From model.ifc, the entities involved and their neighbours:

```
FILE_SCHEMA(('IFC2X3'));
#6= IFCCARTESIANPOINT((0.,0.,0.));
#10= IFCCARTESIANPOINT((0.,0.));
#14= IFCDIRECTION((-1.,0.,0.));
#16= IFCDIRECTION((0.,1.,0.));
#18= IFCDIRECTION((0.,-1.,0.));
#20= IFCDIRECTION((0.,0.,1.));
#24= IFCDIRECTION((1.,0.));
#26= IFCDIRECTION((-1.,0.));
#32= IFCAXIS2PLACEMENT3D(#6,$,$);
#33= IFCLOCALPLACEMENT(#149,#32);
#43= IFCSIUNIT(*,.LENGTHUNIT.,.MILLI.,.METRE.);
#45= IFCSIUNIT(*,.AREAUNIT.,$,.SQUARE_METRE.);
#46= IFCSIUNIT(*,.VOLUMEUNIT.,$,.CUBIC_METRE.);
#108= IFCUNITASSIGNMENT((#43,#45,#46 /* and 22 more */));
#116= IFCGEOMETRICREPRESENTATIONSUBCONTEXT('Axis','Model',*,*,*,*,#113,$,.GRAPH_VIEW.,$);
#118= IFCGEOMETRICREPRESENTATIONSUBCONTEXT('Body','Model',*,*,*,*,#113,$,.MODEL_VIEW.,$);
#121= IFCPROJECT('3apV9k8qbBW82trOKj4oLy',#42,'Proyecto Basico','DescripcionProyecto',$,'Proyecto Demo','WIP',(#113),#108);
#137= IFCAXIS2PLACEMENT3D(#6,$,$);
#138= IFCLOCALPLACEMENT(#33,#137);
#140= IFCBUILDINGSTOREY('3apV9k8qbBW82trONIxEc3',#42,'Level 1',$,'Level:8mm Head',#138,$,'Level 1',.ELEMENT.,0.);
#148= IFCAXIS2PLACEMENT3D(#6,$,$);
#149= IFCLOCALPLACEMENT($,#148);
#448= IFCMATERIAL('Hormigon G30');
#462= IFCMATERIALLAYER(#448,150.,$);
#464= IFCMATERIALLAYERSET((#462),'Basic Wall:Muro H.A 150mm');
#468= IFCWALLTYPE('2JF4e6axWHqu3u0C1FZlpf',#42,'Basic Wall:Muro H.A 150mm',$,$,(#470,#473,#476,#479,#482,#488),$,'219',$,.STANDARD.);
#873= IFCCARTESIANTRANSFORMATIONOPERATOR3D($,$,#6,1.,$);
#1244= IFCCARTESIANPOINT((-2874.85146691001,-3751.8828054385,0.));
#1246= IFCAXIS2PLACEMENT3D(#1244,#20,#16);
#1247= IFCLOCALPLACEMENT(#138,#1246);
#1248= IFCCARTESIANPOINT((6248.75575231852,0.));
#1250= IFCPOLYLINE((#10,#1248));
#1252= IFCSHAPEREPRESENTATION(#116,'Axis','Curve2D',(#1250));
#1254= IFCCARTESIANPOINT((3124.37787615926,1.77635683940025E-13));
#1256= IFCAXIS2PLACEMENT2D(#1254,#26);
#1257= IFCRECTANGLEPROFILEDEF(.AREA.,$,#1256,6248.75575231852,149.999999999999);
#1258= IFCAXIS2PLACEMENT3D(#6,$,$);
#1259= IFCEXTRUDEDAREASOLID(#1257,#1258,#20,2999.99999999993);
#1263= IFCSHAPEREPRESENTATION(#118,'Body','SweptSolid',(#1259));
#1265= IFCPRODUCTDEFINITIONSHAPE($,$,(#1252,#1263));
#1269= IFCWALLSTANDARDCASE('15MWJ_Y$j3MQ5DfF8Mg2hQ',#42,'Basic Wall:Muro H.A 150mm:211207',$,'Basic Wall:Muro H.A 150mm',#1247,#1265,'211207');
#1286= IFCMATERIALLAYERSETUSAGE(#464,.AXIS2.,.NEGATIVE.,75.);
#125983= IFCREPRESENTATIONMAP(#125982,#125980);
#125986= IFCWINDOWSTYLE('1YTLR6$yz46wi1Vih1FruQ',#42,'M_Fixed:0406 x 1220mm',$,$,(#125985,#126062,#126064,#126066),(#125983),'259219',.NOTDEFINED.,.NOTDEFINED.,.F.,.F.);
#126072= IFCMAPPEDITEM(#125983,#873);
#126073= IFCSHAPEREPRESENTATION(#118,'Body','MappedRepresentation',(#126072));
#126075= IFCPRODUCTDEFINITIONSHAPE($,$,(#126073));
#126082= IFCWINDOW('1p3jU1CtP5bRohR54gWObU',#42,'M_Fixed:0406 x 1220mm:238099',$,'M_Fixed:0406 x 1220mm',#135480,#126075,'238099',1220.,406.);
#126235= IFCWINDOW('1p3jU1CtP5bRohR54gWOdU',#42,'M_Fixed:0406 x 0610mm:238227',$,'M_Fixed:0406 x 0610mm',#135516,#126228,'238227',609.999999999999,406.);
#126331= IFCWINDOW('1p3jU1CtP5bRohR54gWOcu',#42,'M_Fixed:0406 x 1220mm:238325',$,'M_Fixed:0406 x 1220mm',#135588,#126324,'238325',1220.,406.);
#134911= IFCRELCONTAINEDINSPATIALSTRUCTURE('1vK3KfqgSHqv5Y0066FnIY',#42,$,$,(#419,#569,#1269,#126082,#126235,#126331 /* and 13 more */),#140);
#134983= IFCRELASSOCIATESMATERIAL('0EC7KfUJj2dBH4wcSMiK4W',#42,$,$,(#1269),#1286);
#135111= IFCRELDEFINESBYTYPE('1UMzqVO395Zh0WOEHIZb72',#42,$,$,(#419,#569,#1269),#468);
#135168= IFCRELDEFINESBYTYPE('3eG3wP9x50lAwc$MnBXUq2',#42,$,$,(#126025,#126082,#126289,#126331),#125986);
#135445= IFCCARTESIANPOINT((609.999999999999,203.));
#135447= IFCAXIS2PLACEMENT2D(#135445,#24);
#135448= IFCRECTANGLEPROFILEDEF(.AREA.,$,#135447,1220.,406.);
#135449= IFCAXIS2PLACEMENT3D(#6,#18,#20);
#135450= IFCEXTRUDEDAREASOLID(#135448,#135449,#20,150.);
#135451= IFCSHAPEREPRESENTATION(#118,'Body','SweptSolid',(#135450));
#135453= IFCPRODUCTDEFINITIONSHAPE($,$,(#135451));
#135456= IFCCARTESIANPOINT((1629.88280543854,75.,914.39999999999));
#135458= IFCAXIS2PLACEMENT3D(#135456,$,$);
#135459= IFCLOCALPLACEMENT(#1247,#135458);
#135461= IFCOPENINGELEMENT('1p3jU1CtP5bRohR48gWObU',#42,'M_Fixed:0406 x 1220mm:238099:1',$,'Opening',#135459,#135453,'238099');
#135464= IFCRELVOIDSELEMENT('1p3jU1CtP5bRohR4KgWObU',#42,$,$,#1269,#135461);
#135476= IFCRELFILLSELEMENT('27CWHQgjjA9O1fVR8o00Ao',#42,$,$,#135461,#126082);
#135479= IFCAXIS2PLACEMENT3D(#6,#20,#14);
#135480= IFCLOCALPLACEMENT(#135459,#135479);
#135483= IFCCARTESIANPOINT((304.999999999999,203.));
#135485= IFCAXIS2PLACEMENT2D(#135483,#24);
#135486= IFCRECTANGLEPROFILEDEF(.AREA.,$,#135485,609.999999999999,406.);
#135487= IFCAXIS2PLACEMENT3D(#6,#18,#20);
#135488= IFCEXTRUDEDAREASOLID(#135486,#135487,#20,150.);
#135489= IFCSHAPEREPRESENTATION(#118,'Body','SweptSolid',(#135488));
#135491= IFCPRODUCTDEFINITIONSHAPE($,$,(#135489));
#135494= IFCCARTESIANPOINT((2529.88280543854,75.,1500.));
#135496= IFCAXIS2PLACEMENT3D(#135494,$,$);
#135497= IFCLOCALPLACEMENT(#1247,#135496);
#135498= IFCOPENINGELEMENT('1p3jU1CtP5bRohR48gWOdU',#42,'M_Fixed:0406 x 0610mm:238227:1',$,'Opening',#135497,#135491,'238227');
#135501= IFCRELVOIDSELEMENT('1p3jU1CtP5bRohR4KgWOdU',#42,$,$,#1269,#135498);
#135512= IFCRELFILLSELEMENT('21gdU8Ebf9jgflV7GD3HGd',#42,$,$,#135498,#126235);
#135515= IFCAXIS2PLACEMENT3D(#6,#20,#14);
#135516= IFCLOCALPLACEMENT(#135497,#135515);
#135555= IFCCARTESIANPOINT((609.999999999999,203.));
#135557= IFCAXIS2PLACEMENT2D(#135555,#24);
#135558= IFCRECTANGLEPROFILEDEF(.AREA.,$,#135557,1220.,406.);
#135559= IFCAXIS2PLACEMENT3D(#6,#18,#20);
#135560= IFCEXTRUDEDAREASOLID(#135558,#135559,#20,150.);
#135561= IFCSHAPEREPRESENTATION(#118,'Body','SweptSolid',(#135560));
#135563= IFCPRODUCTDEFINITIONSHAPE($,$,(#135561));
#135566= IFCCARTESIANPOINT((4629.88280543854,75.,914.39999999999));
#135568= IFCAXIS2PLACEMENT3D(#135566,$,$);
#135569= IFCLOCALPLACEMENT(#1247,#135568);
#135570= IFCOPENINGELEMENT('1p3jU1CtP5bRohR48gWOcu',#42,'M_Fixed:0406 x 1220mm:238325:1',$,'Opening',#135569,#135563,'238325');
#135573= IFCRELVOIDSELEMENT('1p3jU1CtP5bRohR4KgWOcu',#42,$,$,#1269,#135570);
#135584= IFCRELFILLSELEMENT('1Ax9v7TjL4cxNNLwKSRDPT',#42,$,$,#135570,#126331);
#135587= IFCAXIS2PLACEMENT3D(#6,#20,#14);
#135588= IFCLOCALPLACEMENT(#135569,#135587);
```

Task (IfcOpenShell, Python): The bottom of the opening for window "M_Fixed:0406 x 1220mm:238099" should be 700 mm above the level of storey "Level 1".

```python
import numpy as np
import ifcopenshell
import ifcopenshell.api.geometry
import ifcopenshell.geom
import ifcopenshell.util.element
import ifcopenshell.util.placement
import ifcopenshell.util.shape
import ifcopenshell.util.unit

model = ifcopenshell.open("model.ifc")
unit_scale = ifcopenshell.util.unit.calculate_unit_scale(model)

window = model.by_id(126082)
opening = window.FillsVoids[0].RelatingOpeningElement
storey = ifcopenshell.util.element.get_container(window, ifc_class="IfcBuildingStorey")
level = ifcopenshell.util.placement.get_local_placement(storey.ObjectPlacement)[2, 3]

# The opening's origin need not be at the sill, so measure its lowest point.
shape = ifcopenshell.geom.create_shape(ifcopenshell.geom.settings(), opening)
bottom = ifcopenshell.util.shape.get_shape_bottom_elevation(shape, shape.geometry) / unit_scale
dz = level + 0.7 / unit_scale - bottom

shift = np.array([0.0, 0.0, dz])
# The window is placed relative to its opening, so it follows when the opening moves.
matrix = ifcopenshell.util.placement.get_local_placement(opening.ObjectPlacement)
matrix[:3, 3] += shift
ifcopenshell.api.geometry.edit_object_placement(
    model, product=opening, matrix=matrix, is_si=False, should_transform_children=True
)

print(f"moved by {dz * unit_scale:+.3f} m")

model.write("model_v2.ifc")
```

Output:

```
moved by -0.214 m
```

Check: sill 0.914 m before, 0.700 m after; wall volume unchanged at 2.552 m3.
